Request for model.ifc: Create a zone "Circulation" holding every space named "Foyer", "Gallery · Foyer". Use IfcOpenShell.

First a look at what the model holds.

```python
import ifcopenshell

model = ifcopenshell.open("model.ifc")
print(model.schema)
seen = {}
for space in model.by_type("IfcSpace"):
    seen[space.Name] = seen.get(space.Name, 0) + 1
for name, count in sorted(seen.items(), key=str):
    print(count, "x", name)
print("zones:", [z.Name for z in model.by_type("IfcZone")][:20])
```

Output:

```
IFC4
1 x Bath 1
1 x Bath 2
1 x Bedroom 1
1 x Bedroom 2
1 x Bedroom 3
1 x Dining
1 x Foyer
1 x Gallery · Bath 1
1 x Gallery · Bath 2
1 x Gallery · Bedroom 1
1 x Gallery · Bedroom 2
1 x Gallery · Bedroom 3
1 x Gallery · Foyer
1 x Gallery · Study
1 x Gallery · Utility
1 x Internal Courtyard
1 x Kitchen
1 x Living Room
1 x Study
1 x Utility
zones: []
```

```python
import ifcopenshell
import ifcopenshell.api.group
import ifcopenshell.api.root

model = ifcopenshell.open("model.ifc")

names = {"Foyer", "Gallery · Foyer"}
spaces = [s for s in model.by_type("IfcSpace") if s.Name in names]

zone = ifcopenshell.api.root.create_entity(model, ifc_class="IfcZone", name="Circulation")
ifcopenshell.api.group.assign_group(model, products=spaces, group=zone)
print(len(spaces), "spaces in", zone.Name)

model.write("model_v2.ifc")
```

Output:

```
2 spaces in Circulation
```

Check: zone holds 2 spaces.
